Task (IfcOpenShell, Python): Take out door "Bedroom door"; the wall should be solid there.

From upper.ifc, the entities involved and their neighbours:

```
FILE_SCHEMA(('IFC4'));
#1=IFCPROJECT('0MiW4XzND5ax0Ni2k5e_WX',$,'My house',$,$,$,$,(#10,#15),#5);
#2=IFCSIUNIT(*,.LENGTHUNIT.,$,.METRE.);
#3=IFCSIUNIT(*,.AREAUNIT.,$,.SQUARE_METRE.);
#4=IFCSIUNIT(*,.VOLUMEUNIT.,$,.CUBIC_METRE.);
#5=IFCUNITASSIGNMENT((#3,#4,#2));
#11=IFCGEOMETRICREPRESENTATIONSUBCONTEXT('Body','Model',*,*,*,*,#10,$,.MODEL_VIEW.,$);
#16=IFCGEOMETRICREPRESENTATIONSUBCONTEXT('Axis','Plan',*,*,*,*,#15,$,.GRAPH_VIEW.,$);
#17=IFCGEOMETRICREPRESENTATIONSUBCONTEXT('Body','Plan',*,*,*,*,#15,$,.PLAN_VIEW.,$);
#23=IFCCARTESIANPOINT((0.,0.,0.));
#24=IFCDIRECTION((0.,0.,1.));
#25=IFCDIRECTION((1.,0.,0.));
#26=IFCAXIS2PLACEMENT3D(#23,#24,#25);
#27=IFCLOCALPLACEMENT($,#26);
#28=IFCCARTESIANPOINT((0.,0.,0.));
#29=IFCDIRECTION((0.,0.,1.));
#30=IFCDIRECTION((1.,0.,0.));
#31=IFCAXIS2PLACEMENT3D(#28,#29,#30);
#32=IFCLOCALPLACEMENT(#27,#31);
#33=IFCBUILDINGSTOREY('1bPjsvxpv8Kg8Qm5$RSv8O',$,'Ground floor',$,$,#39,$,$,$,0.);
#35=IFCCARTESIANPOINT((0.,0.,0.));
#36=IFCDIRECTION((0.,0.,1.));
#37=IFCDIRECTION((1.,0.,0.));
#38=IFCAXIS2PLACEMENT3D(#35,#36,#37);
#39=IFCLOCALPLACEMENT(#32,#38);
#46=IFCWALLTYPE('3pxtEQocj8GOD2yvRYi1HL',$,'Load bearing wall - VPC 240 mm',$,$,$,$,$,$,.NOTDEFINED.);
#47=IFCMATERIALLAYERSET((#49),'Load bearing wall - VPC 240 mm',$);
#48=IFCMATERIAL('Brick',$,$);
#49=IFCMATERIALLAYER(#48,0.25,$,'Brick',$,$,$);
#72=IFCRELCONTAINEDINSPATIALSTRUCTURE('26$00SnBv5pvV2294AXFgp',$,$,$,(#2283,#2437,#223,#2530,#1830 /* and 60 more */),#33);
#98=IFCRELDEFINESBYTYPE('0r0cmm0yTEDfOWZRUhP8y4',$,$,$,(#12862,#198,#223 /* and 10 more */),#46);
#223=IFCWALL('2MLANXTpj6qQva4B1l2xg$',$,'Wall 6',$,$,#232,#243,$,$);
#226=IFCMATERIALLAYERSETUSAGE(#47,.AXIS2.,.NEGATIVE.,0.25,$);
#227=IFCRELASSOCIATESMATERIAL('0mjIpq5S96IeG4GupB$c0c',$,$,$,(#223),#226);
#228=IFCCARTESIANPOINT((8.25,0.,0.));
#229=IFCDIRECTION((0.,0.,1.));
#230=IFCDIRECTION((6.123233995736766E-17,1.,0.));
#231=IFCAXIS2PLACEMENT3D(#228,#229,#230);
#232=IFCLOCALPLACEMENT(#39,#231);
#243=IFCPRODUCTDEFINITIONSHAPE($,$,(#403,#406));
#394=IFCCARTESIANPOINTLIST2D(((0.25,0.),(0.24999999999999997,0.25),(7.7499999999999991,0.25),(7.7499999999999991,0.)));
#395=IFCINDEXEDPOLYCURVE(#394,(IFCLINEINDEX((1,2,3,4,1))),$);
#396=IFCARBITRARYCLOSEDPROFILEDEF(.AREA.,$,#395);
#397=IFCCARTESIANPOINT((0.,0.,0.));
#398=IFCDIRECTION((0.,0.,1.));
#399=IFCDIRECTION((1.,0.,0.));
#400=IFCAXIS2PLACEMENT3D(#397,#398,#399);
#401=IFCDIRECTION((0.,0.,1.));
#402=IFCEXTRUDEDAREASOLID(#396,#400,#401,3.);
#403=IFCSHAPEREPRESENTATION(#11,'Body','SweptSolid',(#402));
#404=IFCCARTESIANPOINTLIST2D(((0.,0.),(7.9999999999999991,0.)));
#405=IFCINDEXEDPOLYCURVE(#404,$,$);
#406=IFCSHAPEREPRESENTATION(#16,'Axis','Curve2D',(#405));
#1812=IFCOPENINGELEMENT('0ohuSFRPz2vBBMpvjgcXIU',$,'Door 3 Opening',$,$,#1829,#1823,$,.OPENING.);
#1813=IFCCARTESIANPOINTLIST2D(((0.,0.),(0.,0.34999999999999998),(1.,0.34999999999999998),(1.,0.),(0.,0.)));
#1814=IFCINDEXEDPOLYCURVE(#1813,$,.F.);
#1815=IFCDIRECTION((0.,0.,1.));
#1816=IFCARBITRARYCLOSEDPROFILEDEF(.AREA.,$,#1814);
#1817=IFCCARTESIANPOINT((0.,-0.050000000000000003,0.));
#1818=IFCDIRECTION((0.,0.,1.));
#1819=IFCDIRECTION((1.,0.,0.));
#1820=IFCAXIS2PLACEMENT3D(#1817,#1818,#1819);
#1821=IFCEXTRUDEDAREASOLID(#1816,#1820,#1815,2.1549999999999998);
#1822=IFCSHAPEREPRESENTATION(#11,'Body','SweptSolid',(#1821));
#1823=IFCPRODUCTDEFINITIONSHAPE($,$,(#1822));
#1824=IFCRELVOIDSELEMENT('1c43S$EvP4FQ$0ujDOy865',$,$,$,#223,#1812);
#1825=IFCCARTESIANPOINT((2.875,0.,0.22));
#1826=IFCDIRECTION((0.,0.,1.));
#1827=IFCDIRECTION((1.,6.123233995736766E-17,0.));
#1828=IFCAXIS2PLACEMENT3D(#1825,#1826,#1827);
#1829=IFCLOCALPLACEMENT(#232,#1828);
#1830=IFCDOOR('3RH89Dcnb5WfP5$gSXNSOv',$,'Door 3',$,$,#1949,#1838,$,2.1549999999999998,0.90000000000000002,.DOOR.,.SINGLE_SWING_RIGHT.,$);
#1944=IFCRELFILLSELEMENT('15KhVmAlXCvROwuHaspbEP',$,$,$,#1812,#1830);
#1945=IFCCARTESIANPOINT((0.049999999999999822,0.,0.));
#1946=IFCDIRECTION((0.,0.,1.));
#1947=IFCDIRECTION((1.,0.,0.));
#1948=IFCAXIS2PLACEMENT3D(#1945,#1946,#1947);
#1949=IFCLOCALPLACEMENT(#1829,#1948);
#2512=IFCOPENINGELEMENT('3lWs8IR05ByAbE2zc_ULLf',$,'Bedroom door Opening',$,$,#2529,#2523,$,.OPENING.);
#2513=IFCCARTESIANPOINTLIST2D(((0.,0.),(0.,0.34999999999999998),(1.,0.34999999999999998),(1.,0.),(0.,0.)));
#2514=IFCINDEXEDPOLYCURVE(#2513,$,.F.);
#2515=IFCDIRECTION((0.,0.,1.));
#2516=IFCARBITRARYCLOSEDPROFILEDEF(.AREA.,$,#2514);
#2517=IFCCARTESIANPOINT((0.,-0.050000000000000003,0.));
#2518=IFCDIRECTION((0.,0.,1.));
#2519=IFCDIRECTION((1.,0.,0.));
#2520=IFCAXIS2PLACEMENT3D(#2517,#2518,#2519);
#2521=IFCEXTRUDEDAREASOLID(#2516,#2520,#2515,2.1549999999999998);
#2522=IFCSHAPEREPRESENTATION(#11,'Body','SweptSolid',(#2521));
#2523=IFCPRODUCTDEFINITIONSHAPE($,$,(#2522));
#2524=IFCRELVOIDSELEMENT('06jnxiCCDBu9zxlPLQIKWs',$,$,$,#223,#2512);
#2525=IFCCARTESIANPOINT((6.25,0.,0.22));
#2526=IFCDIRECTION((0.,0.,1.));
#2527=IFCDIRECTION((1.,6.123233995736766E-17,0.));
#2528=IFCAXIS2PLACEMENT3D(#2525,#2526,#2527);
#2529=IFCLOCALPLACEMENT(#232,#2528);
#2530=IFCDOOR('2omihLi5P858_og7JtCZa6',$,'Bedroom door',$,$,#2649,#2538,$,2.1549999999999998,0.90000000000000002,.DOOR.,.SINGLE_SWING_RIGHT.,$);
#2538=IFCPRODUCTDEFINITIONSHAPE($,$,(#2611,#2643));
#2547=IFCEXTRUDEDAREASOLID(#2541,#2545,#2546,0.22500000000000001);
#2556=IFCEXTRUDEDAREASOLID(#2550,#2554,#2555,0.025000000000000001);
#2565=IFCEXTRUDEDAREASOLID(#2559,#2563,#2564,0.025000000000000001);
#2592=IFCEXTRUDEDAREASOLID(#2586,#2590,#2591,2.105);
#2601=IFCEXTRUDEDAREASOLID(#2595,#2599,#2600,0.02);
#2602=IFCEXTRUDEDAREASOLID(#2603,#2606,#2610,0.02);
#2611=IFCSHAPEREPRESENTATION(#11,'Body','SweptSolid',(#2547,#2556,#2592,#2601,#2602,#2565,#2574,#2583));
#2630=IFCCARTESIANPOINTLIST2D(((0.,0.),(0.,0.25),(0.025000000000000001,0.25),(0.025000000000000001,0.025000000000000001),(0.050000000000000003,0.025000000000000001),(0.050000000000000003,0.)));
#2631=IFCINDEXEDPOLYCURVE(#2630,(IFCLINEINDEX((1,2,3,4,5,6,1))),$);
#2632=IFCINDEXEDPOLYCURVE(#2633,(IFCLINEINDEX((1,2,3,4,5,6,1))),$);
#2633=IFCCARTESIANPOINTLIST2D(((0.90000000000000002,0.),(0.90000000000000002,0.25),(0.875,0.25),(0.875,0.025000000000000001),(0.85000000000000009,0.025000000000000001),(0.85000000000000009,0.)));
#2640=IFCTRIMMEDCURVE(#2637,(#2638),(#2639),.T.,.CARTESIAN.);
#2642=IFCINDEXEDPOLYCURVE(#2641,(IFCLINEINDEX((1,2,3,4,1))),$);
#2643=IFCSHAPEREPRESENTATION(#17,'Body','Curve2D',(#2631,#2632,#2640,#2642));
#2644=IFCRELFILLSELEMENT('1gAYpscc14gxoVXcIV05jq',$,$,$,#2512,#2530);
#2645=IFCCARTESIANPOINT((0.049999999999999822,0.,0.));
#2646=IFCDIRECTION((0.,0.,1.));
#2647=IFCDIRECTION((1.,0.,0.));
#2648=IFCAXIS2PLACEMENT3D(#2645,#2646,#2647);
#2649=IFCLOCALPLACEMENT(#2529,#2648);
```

```python
import ifcopenshell
import ifcopenshell.api.feature
import ifcopenshell.api.root
import ifcopenshell.geom
import ifcopenshell.util.shape

model = ifcopenshell.open("upper.ifc")
settings = ifcopenshell.geom.settings()


def volume(element):
    """Net volume in cubic metres, openings subtracted."""
    shape = ifcopenshell.geom.create_shape(settings, element)
    return ifcopenshell.util.shape.get_volume(shape.geometry)


door = model.by_guid("2omihLi5P858_og7JtCZa6")
opening = door.FillsVoids[0].RelatingOpeningElement
wall = opening.VoidsElements[0].RelatingBuildingElement
before = volume(wall)

ifcopenshell.api.root.remove_product(model, product=door)
ifcopenshell.api.feature.remove_feature(model, feature=opening)

after = volume(wall)

print(f"wall volume {before:.3f} -> {after:.3f} m3")

model.write("upper_updated.ifc")
```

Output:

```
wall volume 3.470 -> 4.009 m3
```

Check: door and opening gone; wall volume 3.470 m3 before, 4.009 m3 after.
